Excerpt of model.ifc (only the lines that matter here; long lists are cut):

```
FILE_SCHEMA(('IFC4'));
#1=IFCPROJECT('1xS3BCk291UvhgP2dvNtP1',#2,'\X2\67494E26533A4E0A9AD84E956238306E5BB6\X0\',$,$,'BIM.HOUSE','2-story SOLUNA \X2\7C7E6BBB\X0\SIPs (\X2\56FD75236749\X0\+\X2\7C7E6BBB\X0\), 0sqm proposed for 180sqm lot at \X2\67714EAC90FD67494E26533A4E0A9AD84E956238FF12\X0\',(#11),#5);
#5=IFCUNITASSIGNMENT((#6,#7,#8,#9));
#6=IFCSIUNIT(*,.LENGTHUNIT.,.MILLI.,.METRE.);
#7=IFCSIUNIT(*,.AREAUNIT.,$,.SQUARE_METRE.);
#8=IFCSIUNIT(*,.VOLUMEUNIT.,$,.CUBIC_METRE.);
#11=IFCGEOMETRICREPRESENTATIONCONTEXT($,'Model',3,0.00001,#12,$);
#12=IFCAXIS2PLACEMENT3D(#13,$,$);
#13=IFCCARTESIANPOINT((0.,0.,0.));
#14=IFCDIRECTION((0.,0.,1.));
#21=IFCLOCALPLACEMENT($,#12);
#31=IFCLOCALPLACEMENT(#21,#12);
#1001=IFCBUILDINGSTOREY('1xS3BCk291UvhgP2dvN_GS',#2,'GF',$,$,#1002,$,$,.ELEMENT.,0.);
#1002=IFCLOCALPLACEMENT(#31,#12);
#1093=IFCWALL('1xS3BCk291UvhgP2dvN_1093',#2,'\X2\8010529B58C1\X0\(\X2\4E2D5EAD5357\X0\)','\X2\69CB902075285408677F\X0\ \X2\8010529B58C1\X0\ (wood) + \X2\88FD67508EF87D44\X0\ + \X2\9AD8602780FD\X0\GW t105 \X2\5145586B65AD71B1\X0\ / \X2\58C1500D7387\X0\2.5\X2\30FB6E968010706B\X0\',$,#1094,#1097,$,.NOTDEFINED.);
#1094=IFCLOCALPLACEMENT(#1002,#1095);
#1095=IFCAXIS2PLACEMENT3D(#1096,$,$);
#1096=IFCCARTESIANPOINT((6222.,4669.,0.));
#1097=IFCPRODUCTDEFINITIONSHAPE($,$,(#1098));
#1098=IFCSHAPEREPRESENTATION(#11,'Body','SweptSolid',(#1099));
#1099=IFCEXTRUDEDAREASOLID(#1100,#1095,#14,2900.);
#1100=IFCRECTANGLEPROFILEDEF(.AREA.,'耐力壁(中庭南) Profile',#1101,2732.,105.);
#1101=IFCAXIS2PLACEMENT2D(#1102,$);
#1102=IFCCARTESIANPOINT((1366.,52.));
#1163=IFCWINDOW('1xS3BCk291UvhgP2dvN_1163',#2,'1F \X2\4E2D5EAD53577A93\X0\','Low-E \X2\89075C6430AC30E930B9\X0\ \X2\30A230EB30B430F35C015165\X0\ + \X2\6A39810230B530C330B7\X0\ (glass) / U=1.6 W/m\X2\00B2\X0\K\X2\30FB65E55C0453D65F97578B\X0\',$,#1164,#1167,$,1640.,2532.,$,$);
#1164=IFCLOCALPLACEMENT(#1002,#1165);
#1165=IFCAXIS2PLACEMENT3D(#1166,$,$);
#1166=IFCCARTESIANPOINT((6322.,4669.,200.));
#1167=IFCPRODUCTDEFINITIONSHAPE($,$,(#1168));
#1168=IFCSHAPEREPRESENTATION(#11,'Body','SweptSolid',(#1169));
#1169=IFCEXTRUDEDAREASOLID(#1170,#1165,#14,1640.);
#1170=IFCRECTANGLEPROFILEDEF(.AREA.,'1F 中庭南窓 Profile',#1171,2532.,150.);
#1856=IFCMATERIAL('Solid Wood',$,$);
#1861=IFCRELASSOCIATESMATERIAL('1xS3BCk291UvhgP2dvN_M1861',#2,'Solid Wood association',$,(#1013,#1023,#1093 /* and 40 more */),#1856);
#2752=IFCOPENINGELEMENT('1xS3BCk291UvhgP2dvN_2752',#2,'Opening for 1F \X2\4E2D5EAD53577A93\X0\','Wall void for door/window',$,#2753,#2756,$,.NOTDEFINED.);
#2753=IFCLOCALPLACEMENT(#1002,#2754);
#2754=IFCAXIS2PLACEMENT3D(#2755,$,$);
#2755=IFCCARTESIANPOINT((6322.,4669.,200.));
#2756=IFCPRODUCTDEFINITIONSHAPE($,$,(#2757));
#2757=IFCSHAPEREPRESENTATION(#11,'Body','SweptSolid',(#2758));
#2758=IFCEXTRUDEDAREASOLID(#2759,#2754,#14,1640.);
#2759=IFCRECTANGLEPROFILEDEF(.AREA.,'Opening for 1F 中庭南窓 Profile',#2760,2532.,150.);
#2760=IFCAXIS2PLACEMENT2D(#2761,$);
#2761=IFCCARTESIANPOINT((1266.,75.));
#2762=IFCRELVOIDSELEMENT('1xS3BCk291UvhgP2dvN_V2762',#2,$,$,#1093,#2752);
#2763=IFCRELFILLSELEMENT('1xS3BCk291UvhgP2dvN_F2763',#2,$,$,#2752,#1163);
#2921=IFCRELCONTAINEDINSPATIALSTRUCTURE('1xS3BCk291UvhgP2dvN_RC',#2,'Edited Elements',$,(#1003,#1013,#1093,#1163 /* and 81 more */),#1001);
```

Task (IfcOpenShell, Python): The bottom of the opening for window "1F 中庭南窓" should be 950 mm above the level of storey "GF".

```python
import numpy as np
import ifcopenshell
import ifcopenshell.api.geometry
import ifcopenshell.geom
import ifcopenshell.util.element
import ifcopenshell.util.placement
import ifcopenshell.util.shape
import ifcopenshell.util.unit

model = ifcopenshell.open("model.ifc")
unit_scale = ifcopenshell.util.unit.calculate_unit_scale(model)

window = model.by_guid("1xS3BCk291UvhgP2dvN_1163")
opening = window.FillsVoids[0].RelatingOpeningElement
storey = ifcopenshell.util.element.get_container(window, ifc_class="IfcBuildingStorey")
level = ifcopenshell.util.placement.get_local_placement(storey.ObjectPlacement)[2, 3]

# The opening's origin need not be at the sill, so measure its lowest point.
shape = ifcopenshell.geom.create_shape(ifcopenshell.geom.settings(), opening)
bottom = ifcopenshell.util.shape.get_shape_bottom_elevation(shape, shape.geometry) / unit_scale
dz = level + 950.0 - bottom

shift = np.array([0.0, 0.0, dz])
# The window is not placed relative to its opening, so move both.
for product in (opening, window):
    matrix = ifcopenshell.util.placement.get_local_placement(product.ObjectPlacement)
    matrix[:3, 3] += shift
    ifcopenshell.api.geometry.edit_object_placement(model, product=product, matrix=matrix, is_si=False)

print(f"moved by {dz * unit_scale:+.3f} m")

model.write("model_rev.ifc")
```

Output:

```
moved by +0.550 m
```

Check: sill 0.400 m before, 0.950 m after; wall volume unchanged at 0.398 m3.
